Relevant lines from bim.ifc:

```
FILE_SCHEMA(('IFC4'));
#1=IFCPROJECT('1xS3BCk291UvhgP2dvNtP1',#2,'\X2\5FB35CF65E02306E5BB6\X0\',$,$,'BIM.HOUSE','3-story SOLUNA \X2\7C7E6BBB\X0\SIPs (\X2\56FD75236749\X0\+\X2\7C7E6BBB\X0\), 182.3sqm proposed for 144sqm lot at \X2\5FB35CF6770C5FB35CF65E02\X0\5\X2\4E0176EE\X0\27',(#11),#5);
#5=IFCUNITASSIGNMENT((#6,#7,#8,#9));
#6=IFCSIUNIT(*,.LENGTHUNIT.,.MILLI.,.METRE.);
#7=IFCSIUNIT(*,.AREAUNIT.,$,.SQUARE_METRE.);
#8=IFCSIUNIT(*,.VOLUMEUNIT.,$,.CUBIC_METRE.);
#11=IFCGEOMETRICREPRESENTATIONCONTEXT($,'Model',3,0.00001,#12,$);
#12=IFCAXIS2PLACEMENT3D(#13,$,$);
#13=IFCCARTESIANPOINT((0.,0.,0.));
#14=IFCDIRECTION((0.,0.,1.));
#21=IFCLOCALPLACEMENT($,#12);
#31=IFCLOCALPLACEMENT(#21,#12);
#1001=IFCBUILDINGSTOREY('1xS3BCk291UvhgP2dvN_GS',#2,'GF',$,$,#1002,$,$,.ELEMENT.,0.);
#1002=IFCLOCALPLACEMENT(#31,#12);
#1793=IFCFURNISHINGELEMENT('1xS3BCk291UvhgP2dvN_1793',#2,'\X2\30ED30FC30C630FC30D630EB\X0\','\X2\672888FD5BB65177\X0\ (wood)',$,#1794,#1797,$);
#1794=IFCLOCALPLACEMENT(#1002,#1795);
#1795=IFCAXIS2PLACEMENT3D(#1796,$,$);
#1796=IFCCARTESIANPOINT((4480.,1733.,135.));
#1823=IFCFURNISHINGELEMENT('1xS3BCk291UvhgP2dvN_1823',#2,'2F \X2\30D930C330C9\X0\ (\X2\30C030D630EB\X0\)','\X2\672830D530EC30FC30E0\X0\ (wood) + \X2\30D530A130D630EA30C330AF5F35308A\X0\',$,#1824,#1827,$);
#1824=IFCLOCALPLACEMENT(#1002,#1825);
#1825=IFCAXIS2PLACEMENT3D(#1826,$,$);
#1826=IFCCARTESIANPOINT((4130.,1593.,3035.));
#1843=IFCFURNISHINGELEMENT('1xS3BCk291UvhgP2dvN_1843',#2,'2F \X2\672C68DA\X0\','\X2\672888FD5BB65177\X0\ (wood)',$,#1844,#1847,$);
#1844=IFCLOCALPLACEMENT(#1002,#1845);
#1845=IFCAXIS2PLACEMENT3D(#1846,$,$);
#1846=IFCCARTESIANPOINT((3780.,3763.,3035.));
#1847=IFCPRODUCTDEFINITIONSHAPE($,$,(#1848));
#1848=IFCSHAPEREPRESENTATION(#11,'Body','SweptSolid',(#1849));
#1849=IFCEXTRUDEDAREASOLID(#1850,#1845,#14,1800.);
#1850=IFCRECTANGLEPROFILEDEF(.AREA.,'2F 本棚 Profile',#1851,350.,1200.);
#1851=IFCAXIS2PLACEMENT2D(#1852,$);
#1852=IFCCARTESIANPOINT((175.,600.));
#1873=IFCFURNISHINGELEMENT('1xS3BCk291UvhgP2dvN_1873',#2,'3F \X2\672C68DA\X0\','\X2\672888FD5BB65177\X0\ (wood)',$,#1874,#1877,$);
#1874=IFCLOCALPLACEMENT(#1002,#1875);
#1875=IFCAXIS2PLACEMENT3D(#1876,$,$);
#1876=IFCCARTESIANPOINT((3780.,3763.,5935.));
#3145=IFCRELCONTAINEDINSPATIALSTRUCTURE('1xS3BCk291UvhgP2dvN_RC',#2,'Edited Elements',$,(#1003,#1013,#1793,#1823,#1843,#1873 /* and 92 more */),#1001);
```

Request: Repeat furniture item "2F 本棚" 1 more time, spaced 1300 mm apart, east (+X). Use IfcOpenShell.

```python
import numpy as np
import ifcopenshell
import ifcopenshell.api.geometry
import ifcopenshell.api.root
import ifcopenshell.util.element
import ifcopenshell.util.placement
import ifcopenshell.util.unit

model = ifcopenshell.open("bim.ifc")
unit_scale = ifcopenshell.util.unit.calculate_unit_scale(model)


def reuse_history(source, copy):
    """copy_class also copies each property set's owner history, people and application; keep the originals."""
    for rel in copy.IsDefinedBy:
        if rel.is_a("IfcRelDefinesByProperties") and (history := rel.RelatingPropertyDefinition.OwnerHistory):
            rel.RelatingPropertyDefinition.OwnerHistory = source.OwnerHistory
            ifcopenshell.util.element.remove_deep2(model, history)


source = model.by_guid("1xS3BCk291UvhgP2dvN_1843")
base = ifcopenshell.util.placement.get_local_placement(source.ObjectPlacement)
step = np.array([1.0, 0.0, 0.0]) * 1.3 / unit_scale

for i in range(1, 2):
    copy = ifcopenshell.api.root.copy_class(model, product=source)
    copy.Representation = ifcopenshell.util.element.copy_deep(
        model, source.Representation, exclude=["IfcGeometricRepresentationContext", "IfcRepresentationMap"]
    )
    reuse_history(source, copy)
    matrix = base.copy()
    matrix[:3, 3] += i * step
    print("added at", matrix[:3, 3].round(3) + 0.0)
    ifcopenshell.api.geometry.edit_object_placement(model, product=copy, matrix=matrix, is_si=False)

model.write("bim_rev.ifc")
```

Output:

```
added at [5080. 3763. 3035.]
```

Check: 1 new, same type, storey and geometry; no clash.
